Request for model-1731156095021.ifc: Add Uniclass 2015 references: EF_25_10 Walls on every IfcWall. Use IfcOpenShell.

First a look at what the model holds.

```python
import ifcopenshell

model = ifcopenshell.open("model-1731156095021.ifc")
print(model.schema)
print("classifications:", [c.Name for c in model.by_type("IfcClassification")])
for ifc_class in ("IfcDoor", "IfcRoof", "IfcStair", "IfcWall", "IfcWindow"):
    print(ifc_class, len(model.by_type(ifc_class)))
```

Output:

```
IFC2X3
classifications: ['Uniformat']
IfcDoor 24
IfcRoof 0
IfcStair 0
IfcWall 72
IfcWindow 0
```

```python
import ifcopenshell
import ifcopenshell.api.classification

model = ifcopenshell.open("model-1731156095021.ifc")

# IFC2X3 requires Source and Edition and has no link from the project to the system.
system = model.create_entity("IfcClassification", Source="NBS", Edition="2015", Name="Uniclass 2015")

codes = {
    "IfcWall": ("EF_25_10", "Walls"),
}
for ifc_class, (code, name) in codes.items():
    products = model.by_type(ifc_class)
    ifcopenshell.api.classification.add_reference(
        model, products=products, classification=system, identification=code, name=name
    )
    print(code, len(products))

model.write("model-1731156095021_updated.ifc")
```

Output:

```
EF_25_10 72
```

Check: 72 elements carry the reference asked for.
